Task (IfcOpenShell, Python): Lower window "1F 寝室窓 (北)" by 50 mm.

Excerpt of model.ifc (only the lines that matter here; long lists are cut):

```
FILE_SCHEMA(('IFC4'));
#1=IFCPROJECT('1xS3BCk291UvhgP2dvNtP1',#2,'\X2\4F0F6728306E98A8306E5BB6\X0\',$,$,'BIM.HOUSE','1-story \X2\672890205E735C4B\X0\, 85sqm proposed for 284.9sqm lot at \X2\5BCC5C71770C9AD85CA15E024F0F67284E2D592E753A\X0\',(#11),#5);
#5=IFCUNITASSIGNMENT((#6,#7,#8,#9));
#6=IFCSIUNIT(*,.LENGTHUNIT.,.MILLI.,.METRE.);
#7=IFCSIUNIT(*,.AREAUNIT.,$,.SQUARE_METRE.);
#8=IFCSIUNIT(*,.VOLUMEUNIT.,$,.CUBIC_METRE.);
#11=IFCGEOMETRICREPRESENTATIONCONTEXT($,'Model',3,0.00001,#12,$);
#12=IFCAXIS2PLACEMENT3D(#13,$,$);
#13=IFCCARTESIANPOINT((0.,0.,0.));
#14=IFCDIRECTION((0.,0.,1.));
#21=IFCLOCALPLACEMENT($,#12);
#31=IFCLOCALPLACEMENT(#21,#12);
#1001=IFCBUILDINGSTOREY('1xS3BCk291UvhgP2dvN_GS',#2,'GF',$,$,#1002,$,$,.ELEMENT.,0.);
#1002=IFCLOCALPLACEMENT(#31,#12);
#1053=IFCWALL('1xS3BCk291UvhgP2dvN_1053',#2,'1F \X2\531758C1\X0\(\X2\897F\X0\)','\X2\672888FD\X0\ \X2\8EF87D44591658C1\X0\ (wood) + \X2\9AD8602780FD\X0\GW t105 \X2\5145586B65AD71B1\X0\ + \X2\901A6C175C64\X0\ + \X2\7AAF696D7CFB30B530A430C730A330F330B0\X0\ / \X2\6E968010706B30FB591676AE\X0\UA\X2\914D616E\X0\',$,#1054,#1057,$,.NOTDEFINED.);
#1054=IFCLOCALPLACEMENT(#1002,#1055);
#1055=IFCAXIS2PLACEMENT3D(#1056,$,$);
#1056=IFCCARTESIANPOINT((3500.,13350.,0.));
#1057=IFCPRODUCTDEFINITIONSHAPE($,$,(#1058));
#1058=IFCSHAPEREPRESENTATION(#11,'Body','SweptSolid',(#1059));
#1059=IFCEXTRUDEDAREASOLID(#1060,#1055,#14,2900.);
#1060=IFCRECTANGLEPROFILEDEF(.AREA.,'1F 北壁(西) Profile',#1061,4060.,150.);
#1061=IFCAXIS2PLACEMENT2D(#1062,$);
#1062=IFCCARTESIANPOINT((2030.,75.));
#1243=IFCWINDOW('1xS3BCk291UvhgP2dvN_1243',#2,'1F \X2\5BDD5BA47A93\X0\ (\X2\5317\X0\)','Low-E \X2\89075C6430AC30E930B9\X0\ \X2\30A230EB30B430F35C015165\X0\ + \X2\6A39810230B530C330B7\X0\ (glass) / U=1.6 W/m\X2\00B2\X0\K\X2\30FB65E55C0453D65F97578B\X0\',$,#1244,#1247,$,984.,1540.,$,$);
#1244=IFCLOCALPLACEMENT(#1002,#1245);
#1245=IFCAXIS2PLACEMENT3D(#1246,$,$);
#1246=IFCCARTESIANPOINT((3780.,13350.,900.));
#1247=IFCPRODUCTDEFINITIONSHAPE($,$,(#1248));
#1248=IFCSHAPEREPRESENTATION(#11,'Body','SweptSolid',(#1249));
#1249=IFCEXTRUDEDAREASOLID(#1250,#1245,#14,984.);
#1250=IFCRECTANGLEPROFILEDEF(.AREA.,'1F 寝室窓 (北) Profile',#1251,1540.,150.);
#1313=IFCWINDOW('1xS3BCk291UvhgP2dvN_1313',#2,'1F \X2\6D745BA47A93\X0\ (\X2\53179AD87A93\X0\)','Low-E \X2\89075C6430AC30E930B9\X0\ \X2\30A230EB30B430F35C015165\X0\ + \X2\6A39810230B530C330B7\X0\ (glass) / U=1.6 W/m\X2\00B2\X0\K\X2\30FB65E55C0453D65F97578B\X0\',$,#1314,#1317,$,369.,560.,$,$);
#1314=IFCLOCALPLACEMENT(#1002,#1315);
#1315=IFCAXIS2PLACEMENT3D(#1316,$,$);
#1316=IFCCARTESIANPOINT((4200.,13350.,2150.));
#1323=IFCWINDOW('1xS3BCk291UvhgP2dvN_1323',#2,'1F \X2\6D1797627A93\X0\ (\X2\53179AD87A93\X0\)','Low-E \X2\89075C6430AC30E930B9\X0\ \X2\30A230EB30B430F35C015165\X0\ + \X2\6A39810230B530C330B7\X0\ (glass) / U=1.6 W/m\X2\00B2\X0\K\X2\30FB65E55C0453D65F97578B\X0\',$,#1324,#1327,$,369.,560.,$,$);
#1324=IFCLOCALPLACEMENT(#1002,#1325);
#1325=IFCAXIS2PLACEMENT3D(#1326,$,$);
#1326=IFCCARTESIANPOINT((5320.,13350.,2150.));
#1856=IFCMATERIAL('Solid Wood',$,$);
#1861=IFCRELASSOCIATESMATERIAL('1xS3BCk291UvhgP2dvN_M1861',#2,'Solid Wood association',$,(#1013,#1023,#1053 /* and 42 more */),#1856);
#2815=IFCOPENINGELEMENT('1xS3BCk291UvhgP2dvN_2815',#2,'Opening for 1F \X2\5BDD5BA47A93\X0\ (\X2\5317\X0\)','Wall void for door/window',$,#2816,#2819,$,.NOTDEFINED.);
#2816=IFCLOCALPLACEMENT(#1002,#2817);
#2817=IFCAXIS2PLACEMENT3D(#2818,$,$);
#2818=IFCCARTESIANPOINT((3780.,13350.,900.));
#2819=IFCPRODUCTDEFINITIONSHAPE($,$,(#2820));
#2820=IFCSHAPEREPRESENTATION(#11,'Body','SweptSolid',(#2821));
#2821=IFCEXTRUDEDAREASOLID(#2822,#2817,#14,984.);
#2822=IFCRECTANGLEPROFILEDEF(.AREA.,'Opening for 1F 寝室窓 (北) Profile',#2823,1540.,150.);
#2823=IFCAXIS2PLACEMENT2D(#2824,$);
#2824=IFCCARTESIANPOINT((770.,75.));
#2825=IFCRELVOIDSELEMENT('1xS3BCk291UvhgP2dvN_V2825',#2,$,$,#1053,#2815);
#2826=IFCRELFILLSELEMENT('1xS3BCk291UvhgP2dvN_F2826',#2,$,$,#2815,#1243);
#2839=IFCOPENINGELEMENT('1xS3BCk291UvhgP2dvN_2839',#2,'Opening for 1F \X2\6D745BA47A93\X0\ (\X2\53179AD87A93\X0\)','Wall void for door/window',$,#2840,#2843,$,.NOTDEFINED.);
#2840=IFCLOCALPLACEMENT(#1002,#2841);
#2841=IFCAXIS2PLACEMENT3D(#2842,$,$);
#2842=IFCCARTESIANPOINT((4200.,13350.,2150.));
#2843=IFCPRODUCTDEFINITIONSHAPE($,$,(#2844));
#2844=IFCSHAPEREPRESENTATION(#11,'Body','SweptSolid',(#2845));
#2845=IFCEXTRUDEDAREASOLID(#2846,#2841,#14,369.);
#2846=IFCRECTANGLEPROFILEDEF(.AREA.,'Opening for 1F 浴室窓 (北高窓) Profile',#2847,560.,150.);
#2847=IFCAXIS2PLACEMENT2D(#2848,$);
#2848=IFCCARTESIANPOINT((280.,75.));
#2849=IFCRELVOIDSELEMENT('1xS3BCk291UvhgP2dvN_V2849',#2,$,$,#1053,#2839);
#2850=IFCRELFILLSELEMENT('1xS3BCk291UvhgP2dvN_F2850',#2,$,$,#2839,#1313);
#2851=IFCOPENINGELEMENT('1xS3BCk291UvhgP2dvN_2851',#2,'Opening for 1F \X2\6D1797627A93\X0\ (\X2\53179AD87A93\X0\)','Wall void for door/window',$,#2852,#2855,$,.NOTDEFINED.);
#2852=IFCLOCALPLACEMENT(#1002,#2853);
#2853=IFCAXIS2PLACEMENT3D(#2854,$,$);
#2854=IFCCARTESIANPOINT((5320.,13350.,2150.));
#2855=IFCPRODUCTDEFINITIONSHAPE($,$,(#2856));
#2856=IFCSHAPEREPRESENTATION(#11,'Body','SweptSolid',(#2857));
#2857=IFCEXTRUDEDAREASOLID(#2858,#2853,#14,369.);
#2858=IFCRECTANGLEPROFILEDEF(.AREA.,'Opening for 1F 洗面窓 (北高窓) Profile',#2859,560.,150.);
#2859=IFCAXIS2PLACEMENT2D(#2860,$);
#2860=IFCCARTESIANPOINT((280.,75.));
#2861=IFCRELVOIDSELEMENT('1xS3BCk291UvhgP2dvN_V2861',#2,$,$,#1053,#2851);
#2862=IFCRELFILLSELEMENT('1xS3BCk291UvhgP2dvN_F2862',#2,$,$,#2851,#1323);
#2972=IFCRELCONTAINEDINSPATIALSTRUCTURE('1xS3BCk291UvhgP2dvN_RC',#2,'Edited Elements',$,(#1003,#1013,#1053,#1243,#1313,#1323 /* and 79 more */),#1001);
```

```python
import numpy as np
import ifcopenshell
import ifcopenshell.api.geometry
import ifcopenshell.util.placement
import ifcopenshell.util.unit

model = ifcopenshell.open("model.ifc")
unit_scale = ifcopenshell.util.unit.calculate_unit_scale(model)

window = model.by_id(1243)
opening = window.FillsVoids[0].RelatingOpeningElement
dz = -50.0

shift = np.array([0.0, 0.0, dz])
# The window is not placed relative to its opening, so move both.
for product in (opening, window):
    matrix = ifcopenshell.util.placement.get_local_placement(product.ObjectPlacement)
    matrix[:3, 3] += shift
    ifcopenshell.api.geometry.edit_object_placement(model, product=product, matrix=matrix, is_si=False)

print(f"moved by {dz * unit_scale:+.3f} m")

model.write("model_edited.ifc")
```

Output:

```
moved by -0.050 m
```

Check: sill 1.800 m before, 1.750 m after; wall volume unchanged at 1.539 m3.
